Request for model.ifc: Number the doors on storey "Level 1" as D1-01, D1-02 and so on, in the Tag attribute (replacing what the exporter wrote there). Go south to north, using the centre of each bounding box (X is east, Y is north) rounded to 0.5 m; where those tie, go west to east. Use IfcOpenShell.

First a look at what the model holds.

```python
import ifcopenshell
import ifcopenshell.util.element
import ifcopenshell.util.placement

model = ifcopenshell.open("model.ifc")
print(model.schema)
storey = next(s for s in model.by_type("IfcBuildingStorey") if s.Name == "Level 1")
doors = [e for e in ifcopenshell.util.element.get_decomposition(storey) if e.is_a("IfcDoor")]
for e in sorted(doors, key=lambda e: e.id()):
    origin = ifcopenshell.util.placement.get_local_placement(e.ObjectPlacement)[:3, 3]
    print(e.id(), e.Tag, e.Name, origin.round(2) + 0.0, sep=" | ")
```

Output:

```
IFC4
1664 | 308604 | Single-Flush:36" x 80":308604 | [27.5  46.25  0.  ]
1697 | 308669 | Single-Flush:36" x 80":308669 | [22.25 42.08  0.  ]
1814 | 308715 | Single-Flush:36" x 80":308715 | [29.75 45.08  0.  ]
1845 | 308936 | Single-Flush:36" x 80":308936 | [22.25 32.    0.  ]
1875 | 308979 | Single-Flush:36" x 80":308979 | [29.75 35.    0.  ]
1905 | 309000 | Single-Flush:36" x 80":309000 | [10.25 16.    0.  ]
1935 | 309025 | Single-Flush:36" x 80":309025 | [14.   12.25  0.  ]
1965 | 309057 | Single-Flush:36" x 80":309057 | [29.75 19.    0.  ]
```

```python
import ifcopenshell
import ifcopenshell.geom
import ifcopenshell.util.element
import ifcopenshell.util.shape

model = ifcopenshell.open("model.ifc")
settings = ifcopenshell.geom.settings()
settings.set("use-world-coords", True)


def centre(element):
    shape = ifcopenshell.geom.create_shape(settings, element)
    return ifcopenshell.util.shape.get_bbox_centroid(shape.geometry)


storey = next(s for s in model.by_type("IfcBuildingStorey") if s.Name == "Level 1")
doors = [e for e in ifcopenshell.util.element.get_decomposition(storey) if e.is_a("IfcDoor")]

# Insertion points can sit at a corner or the storey origin, so sort by the geometry (in metres).
centres = {e: centre(e) for e in doors}
doors.sort(key=lambda e: (round(centres[e][1] / 0.5), centres[e][0]))

for i, e in enumerate(doors, start=1):
    number = f"D1-{i:02d}"
    e.Tag = number
    print(e.id(), number)

model.write("model-out.ifc")
```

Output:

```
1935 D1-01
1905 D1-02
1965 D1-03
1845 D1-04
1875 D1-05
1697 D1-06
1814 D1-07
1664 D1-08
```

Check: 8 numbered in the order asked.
